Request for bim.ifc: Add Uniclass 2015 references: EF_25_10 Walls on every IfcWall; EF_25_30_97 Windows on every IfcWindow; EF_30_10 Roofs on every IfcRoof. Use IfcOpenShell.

First a look at what the model holds.

```python
import ifcopenshell

model = ifcopenshell.open("bim.ifc")
print(model.schema)
print("classifications:", [c.Name for c in model.by_type("IfcClassification")])
for ifc_class in ("IfcDoor", "IfcRoof", "IfcStair", "IfcWall", "IfcWindow"):
    print(ifc_class, len(model.by_type(ifc_class)))
```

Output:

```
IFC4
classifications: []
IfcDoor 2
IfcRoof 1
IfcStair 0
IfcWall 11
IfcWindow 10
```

```python
import ifcopenshell
import ifcopenshell.api.classification

model = ifcopenshell.open("bim.ifc")

system = ifcopenshell.api.classification.add_classification(model, classification="Uniclass 2015")

codes = {
    "IfcWall": ("EF_25_10", "Walls"),
    "IfcWindow": ("EF_25_30_97", "Windows"),
    "IfcRoof": ("EF_30_10", "Roofs"),
}
for ifc_class, (code, name) in codes.items():
    products = model.by_type(ifc_class)
    ifcopenshell.api.classification.add_reference(
        model, products=products, classification=system, identification=code, name=name
    )
    print(code, len(products))

model.write("bim_v2.ifc")
```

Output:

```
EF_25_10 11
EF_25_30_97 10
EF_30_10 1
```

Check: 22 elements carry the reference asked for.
